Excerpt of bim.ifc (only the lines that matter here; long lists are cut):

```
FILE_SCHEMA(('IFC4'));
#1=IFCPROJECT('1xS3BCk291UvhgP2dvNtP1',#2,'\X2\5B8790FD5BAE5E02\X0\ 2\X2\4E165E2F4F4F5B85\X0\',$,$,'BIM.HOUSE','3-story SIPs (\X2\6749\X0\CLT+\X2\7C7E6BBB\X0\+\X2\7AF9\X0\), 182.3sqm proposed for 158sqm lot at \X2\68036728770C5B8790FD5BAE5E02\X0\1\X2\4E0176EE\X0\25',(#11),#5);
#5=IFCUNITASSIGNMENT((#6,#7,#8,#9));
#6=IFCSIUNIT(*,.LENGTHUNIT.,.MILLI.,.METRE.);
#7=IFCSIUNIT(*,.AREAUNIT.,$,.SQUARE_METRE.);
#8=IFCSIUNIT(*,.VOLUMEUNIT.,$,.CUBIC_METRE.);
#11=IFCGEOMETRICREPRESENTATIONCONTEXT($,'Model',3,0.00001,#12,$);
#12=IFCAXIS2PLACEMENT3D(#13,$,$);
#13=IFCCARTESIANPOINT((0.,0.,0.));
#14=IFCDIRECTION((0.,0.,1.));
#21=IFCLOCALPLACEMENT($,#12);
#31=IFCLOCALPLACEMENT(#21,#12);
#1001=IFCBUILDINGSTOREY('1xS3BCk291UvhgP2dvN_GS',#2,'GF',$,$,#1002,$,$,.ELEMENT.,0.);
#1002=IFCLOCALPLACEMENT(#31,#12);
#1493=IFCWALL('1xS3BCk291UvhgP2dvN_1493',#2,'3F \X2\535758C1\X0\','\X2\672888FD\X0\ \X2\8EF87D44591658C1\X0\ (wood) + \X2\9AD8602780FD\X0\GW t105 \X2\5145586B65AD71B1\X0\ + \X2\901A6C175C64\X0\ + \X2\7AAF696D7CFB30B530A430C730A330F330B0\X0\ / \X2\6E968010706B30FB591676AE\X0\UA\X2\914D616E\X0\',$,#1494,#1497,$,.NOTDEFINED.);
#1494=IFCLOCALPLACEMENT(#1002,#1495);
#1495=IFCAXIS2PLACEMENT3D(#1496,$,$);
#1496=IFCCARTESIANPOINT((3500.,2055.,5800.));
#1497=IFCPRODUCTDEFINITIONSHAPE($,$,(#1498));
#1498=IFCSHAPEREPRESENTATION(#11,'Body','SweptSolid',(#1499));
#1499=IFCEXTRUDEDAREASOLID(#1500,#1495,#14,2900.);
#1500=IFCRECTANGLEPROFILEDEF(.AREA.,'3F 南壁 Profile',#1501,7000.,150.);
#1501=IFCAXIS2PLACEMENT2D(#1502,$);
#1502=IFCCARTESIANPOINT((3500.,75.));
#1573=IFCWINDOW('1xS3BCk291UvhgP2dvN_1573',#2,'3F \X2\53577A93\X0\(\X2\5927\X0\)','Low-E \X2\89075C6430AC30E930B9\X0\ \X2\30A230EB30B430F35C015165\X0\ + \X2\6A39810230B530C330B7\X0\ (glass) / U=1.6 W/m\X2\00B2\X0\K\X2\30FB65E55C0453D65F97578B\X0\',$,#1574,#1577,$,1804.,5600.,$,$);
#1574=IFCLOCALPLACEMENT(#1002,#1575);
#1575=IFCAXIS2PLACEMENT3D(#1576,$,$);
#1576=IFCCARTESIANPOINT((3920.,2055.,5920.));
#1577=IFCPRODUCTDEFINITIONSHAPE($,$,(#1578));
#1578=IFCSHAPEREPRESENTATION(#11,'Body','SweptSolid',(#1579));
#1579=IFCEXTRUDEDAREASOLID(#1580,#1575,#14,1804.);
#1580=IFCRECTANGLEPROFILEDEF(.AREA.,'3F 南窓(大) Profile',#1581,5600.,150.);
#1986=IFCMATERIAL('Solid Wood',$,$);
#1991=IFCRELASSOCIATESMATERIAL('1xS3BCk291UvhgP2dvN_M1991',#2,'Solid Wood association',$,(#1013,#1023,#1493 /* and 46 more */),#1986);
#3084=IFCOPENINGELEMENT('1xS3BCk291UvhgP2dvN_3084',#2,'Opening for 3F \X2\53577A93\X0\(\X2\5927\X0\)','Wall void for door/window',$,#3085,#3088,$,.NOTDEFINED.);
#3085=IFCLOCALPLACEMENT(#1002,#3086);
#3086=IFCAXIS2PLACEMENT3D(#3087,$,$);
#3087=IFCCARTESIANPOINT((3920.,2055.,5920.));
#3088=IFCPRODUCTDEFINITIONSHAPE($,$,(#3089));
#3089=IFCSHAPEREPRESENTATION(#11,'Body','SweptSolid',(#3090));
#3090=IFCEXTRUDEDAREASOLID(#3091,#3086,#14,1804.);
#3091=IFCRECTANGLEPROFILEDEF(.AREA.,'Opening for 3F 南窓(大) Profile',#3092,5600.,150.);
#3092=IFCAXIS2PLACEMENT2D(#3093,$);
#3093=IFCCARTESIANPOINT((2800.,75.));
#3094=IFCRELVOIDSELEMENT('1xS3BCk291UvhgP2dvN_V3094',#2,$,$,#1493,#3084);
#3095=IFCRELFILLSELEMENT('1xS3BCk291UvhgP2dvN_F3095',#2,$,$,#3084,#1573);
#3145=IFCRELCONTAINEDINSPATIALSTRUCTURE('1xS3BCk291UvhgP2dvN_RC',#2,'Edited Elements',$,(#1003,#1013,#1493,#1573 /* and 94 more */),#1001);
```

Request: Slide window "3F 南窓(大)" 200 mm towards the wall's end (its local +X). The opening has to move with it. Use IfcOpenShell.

```python
import ifcopenshell
import ifcopenshell.api.geometry
import ifcopenshell.util.placement

model = ifcopenshell.open("bim.ifc")

window = model.by_id(1573)
opening = window.FillsVoids[0].RelatingOpeningElement
wall = opening.VoidsElements[0].RelatingBuildingElement

wall_matrix = ifcopenshell.util.placement.get_local_placement(wall.ObjectPlacement)
shift = wall_matrix[:3, 0] * 200.0
before = ifcopenshell.util.placement.get_local_placement(window.ObjectPlacement)[:3, 3].copy()

# The window is not placed relative to its opening, so move both.
for product in (opening, window):
    matrix = ifcopenshell.util.placement.get_local_placement(product.ObjectPlacement)
    matrix[:3, 3] += shift
    ifcopenshell.api.geometry.edit_object_placement(model, product=product, matrix=matrix, is_si=False)

after = ifcopenshell.util.placement.get_local_placement(window.ObjectPlacement)[:3, 3]
print("window moved by", (after - before).round(3) + 0.0)

model.write("bim_edited.ifc")
```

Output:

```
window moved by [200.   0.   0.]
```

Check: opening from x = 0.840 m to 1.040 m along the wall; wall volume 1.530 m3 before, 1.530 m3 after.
